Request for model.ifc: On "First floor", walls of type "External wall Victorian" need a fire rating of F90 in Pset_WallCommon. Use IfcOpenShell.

First a look at what the model holds.

```python
import ifcopenshell
import ifcopenshell.util.element

model = ifcopenshell.open("model.ifc")
print(model.schema)
storey = next(s for s in model.by_type("IfcBuildingStorey") if s.Name == "First floor")
walls = [e for e in ifcopenshell.util.element.get_decomposition(storey) if e.is_a("IfcWall")]
seen = {}
for e in walls:
    element_type = ifcopenshell.util.element.get_type(e)
    key = (element_type.Name if element_type != e and element_type else None, ifcopenshell.util.element.get_pset(e, "Pset_WallCommon", "FireRating"))
    seen[key] = seen.get(key, 0) + 1
for (name, value), count in sorted(seen.items(), key=str):
    print(count, "x", name, "|", value)
```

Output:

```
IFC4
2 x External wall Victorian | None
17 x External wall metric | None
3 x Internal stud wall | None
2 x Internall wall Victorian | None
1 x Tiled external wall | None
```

```python
import ifcopenshell
import ifcopenshell.api.pset
import ifcopenshell.util.element

model = ifcopenshell.open("model.ifc")

storey = next(s for s in model.by_type("IfcBuildingStorey") if s.Name == "First floor")
walls = [e for e in ifcopenshell.util.element.get_decomposition(storey) if e.is_a("IfcWall")]

count = 0
for e in walls:
    element_type = ifcopenshell.util.element.get_type(e)
    if element_type in (None, e) or element_type.Name != "External wall Victorian":
        continue
    # add_pset returns the element's existing set when there is one.
    pset = ifcopenshell.api.pset.add_pset(model, product=e, name="Pset_WallCommon")
    ifcopenshell.api.pset.edit_pset(model, pset=pset, properties={"FireRating": "F90"})
    count += 1

print(count, "walls updated")

model.write("model_updated.ifc")
```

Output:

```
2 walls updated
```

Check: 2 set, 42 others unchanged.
